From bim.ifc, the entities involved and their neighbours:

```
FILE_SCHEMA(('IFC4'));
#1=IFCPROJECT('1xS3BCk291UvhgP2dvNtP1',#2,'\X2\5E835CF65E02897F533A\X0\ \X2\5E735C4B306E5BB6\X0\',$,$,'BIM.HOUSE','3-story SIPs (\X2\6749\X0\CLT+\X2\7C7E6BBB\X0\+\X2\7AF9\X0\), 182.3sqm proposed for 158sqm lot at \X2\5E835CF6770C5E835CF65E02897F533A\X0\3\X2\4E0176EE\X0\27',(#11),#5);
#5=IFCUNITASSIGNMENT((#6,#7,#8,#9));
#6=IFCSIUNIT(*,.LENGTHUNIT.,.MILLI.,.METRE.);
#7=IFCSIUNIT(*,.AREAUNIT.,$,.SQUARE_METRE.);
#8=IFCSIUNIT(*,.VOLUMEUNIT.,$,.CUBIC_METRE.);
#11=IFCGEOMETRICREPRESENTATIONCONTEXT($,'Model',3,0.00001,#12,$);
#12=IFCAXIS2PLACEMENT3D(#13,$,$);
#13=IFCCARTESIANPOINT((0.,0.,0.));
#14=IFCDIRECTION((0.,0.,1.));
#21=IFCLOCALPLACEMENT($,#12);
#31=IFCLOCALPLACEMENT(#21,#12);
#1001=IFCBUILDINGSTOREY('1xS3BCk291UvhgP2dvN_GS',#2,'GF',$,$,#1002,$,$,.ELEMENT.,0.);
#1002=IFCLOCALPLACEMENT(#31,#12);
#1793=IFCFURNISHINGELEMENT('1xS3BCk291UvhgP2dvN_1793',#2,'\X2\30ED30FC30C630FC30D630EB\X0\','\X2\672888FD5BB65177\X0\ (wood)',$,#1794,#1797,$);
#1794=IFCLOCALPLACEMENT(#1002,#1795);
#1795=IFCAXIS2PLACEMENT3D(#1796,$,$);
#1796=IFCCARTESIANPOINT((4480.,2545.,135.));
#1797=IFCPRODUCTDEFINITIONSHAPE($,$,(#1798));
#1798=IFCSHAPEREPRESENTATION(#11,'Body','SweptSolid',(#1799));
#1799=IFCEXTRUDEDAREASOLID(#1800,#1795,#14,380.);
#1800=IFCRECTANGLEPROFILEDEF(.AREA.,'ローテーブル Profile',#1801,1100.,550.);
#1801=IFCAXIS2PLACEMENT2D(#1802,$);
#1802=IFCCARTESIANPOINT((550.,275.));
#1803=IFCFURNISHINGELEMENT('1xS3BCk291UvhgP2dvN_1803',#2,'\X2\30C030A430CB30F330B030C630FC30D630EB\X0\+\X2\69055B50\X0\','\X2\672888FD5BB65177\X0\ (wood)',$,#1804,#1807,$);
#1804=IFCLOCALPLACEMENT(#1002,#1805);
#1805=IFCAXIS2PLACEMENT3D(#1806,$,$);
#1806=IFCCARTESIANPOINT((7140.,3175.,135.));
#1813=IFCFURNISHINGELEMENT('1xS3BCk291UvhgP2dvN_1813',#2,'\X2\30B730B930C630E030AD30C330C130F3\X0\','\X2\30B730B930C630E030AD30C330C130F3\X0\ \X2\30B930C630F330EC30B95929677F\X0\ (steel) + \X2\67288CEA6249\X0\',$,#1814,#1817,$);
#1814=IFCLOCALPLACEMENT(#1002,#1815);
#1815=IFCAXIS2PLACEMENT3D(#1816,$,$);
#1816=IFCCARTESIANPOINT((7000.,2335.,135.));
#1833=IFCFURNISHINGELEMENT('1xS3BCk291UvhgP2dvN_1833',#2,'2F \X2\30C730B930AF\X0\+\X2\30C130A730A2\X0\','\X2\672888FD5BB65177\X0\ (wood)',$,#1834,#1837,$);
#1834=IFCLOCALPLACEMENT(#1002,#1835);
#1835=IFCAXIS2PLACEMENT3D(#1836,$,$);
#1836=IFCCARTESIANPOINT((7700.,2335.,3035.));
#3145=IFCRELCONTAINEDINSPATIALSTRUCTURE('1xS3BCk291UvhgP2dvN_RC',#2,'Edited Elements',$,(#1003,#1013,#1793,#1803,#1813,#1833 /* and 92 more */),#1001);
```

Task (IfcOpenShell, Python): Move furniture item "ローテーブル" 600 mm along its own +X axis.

```python
import ifcopenshell
import ifcopenshell.api.geometry
import ifcopenshell.util.placement
import ifcopenshell.util.unit

model = ifcopenshell.open("bim.ifc")
unit_scale = ifcopenshell.util.unit.calculate_unit_scale(model)

item = model.by_guid("1xS3BCk291UvhgP2dvN_1793")
matrix = ifcopenshell.util.placement.get_local_placement(item.ObjectPlacement)
matrix[:3, 3] += matrix[:3, 0] * 0.6 / unit_scale
ifcopenshell.api.geometry.edit_object_placement(model, product=item, matrix=matrix, is_si=False)

print(ifcopenshell.util.placement.get_local_placement(item.ObjectPlacement).round(3) + 0.0)

model.write("bim_v2.ifc")
```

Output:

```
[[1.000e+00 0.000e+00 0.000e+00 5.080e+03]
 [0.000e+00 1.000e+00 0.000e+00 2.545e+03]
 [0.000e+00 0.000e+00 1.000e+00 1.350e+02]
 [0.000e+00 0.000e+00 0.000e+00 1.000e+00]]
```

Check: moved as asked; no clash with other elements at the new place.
